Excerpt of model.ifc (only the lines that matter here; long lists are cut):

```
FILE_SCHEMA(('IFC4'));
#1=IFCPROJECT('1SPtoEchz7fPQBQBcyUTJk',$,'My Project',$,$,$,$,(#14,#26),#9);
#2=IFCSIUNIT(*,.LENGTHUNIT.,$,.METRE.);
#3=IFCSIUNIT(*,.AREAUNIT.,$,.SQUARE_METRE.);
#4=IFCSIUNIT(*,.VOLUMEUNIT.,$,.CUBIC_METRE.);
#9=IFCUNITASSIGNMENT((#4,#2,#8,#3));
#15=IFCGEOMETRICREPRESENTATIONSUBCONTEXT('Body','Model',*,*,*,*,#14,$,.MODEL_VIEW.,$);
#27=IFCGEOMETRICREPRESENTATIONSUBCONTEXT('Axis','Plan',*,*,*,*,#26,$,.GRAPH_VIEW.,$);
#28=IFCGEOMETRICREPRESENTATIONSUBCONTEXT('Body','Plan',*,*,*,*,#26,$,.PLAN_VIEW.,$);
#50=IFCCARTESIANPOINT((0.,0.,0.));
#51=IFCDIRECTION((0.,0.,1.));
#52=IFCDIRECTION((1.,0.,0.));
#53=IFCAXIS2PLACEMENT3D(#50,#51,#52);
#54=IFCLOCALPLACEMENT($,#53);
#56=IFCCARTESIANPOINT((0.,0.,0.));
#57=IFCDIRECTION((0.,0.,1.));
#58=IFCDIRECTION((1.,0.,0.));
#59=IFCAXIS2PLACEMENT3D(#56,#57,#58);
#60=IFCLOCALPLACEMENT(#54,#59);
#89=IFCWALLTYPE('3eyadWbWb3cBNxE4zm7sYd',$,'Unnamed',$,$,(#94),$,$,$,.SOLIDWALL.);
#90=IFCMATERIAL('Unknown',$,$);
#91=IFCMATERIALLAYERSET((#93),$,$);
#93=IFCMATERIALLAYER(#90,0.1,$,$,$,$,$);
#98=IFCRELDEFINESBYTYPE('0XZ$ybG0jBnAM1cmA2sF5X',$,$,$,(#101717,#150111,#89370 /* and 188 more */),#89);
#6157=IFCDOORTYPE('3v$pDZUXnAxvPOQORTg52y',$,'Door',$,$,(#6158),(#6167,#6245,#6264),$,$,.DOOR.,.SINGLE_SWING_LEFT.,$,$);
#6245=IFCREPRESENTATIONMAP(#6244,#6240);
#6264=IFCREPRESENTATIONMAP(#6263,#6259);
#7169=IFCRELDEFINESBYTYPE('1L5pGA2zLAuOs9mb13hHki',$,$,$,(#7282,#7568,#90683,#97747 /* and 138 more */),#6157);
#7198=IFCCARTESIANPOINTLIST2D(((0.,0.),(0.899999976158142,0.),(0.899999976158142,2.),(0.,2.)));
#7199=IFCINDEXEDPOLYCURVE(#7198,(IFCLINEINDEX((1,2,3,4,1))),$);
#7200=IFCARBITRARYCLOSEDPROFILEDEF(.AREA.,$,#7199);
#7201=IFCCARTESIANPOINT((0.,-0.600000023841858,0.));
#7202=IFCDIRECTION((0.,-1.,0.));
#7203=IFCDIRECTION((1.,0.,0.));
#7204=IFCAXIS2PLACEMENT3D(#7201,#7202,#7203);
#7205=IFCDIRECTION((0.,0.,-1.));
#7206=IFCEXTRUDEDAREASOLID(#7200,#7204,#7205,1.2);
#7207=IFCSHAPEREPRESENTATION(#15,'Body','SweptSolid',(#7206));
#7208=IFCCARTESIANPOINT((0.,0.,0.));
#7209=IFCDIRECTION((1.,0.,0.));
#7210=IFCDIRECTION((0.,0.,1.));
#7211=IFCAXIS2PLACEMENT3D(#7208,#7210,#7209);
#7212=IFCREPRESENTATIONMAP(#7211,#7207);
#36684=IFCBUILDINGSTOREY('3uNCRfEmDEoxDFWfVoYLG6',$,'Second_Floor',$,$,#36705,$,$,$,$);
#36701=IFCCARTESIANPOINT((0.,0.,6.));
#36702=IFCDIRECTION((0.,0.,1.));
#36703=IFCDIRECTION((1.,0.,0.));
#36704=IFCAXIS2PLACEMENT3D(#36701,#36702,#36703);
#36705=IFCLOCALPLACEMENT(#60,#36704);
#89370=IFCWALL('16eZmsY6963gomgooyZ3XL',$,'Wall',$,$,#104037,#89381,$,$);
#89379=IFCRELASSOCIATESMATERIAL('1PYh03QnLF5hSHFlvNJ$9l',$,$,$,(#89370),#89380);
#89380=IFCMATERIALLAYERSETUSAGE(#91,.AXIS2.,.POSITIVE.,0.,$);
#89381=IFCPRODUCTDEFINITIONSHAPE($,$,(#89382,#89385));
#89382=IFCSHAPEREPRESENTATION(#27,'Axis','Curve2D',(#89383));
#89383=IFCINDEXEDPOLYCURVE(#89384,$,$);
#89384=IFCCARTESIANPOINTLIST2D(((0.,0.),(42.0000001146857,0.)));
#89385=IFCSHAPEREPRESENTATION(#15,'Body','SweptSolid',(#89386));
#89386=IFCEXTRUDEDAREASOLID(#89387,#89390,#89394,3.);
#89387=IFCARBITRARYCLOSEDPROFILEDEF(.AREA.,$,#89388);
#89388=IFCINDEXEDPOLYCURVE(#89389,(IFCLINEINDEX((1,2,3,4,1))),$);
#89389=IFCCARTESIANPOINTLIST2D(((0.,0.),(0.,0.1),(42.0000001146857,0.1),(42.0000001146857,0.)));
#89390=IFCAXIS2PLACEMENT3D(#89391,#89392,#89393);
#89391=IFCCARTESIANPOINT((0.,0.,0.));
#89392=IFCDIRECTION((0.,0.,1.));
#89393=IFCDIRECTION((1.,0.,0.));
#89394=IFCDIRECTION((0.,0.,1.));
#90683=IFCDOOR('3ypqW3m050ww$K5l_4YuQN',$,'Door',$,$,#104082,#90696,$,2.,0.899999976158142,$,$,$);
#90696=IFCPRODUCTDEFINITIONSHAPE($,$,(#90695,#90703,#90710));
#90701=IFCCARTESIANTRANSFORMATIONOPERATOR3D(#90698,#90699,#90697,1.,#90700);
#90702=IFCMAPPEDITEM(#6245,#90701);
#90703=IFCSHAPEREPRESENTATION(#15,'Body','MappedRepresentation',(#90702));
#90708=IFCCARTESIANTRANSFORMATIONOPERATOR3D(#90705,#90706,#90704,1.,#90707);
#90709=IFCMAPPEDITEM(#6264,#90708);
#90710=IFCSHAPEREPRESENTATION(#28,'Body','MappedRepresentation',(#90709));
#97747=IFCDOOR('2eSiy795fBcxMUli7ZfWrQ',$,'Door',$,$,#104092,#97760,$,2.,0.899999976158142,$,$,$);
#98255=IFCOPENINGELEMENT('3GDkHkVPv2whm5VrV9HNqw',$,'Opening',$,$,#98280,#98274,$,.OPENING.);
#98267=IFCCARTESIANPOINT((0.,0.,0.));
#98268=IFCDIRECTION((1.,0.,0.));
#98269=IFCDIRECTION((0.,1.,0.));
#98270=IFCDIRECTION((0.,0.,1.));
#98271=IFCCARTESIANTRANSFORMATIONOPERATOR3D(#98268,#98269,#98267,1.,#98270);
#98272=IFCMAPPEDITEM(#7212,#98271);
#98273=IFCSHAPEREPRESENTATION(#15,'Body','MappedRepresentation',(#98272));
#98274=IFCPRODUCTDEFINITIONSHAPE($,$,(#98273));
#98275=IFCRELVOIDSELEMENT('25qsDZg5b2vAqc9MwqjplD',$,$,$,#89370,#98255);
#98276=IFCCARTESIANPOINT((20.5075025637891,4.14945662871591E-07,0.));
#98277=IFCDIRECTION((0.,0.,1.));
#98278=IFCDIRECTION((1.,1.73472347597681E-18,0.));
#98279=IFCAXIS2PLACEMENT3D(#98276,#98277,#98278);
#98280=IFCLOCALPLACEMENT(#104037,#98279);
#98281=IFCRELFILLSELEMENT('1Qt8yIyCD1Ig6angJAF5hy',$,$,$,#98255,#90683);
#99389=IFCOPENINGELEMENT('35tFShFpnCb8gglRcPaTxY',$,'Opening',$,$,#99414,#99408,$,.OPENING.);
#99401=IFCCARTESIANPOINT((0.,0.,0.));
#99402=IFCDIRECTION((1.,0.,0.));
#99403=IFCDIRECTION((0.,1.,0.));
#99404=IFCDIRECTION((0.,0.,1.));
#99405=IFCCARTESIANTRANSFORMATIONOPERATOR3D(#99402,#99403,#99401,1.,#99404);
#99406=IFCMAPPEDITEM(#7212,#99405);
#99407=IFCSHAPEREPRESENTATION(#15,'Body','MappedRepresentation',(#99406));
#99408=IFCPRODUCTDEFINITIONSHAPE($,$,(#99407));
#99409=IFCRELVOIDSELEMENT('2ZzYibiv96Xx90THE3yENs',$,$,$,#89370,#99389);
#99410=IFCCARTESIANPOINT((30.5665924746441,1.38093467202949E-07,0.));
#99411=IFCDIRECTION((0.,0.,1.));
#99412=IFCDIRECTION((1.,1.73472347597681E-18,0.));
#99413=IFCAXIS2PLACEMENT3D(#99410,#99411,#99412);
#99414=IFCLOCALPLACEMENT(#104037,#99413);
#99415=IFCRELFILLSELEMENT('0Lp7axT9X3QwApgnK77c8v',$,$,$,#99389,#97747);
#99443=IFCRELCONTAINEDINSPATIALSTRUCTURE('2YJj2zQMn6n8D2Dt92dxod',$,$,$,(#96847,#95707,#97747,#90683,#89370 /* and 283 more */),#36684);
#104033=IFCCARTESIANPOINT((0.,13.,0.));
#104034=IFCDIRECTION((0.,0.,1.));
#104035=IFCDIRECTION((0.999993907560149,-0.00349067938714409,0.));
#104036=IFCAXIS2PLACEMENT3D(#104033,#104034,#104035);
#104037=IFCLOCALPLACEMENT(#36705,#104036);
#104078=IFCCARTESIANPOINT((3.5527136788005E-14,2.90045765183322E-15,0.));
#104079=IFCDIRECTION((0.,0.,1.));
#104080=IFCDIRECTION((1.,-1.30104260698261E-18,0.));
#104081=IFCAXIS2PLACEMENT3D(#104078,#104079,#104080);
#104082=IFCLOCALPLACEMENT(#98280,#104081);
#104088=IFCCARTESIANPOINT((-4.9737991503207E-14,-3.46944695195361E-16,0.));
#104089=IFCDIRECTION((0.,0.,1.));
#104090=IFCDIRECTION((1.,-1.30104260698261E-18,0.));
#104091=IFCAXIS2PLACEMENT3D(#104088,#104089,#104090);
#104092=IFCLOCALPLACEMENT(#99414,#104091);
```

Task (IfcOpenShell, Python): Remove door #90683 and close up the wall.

```python
import ifcopenshell
import ifcopenshell.api.feature
import ifcopenshell.api.root
import ifcopenshell.geom
import ifcopenshell.util.shape

model = ifcopenshell.open("model.ifc")
settings = ifcopenshell.geom.settings()


def volume(element):
    """Net volume in cubic metres, openings subtracted."""
    shape = ifcopenshell.geom.create_shape(settings, element)
    return ifcopenshell.util.shape.get_volume(shape.geometry)


door = model.by_guid("3ypqW3m050ww$K5l_4YuQN")
opening = door.FillsVoids[0].RelatingOpeningElement
wall = opening.VoidsElements[0].RelatingBuildingElement
before = volume(wall)

ifcopenshell.api.root.remove_product(model, product=door)
ifcopenshell.api.feature.remove_feature(model, feature=opening)

after = volume(wall)

print(f"wall volume {before:.3f} -> {after:.3f} m3")

model.write("model-out.ifc")
```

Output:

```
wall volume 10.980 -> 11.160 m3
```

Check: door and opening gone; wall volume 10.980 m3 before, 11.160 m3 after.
